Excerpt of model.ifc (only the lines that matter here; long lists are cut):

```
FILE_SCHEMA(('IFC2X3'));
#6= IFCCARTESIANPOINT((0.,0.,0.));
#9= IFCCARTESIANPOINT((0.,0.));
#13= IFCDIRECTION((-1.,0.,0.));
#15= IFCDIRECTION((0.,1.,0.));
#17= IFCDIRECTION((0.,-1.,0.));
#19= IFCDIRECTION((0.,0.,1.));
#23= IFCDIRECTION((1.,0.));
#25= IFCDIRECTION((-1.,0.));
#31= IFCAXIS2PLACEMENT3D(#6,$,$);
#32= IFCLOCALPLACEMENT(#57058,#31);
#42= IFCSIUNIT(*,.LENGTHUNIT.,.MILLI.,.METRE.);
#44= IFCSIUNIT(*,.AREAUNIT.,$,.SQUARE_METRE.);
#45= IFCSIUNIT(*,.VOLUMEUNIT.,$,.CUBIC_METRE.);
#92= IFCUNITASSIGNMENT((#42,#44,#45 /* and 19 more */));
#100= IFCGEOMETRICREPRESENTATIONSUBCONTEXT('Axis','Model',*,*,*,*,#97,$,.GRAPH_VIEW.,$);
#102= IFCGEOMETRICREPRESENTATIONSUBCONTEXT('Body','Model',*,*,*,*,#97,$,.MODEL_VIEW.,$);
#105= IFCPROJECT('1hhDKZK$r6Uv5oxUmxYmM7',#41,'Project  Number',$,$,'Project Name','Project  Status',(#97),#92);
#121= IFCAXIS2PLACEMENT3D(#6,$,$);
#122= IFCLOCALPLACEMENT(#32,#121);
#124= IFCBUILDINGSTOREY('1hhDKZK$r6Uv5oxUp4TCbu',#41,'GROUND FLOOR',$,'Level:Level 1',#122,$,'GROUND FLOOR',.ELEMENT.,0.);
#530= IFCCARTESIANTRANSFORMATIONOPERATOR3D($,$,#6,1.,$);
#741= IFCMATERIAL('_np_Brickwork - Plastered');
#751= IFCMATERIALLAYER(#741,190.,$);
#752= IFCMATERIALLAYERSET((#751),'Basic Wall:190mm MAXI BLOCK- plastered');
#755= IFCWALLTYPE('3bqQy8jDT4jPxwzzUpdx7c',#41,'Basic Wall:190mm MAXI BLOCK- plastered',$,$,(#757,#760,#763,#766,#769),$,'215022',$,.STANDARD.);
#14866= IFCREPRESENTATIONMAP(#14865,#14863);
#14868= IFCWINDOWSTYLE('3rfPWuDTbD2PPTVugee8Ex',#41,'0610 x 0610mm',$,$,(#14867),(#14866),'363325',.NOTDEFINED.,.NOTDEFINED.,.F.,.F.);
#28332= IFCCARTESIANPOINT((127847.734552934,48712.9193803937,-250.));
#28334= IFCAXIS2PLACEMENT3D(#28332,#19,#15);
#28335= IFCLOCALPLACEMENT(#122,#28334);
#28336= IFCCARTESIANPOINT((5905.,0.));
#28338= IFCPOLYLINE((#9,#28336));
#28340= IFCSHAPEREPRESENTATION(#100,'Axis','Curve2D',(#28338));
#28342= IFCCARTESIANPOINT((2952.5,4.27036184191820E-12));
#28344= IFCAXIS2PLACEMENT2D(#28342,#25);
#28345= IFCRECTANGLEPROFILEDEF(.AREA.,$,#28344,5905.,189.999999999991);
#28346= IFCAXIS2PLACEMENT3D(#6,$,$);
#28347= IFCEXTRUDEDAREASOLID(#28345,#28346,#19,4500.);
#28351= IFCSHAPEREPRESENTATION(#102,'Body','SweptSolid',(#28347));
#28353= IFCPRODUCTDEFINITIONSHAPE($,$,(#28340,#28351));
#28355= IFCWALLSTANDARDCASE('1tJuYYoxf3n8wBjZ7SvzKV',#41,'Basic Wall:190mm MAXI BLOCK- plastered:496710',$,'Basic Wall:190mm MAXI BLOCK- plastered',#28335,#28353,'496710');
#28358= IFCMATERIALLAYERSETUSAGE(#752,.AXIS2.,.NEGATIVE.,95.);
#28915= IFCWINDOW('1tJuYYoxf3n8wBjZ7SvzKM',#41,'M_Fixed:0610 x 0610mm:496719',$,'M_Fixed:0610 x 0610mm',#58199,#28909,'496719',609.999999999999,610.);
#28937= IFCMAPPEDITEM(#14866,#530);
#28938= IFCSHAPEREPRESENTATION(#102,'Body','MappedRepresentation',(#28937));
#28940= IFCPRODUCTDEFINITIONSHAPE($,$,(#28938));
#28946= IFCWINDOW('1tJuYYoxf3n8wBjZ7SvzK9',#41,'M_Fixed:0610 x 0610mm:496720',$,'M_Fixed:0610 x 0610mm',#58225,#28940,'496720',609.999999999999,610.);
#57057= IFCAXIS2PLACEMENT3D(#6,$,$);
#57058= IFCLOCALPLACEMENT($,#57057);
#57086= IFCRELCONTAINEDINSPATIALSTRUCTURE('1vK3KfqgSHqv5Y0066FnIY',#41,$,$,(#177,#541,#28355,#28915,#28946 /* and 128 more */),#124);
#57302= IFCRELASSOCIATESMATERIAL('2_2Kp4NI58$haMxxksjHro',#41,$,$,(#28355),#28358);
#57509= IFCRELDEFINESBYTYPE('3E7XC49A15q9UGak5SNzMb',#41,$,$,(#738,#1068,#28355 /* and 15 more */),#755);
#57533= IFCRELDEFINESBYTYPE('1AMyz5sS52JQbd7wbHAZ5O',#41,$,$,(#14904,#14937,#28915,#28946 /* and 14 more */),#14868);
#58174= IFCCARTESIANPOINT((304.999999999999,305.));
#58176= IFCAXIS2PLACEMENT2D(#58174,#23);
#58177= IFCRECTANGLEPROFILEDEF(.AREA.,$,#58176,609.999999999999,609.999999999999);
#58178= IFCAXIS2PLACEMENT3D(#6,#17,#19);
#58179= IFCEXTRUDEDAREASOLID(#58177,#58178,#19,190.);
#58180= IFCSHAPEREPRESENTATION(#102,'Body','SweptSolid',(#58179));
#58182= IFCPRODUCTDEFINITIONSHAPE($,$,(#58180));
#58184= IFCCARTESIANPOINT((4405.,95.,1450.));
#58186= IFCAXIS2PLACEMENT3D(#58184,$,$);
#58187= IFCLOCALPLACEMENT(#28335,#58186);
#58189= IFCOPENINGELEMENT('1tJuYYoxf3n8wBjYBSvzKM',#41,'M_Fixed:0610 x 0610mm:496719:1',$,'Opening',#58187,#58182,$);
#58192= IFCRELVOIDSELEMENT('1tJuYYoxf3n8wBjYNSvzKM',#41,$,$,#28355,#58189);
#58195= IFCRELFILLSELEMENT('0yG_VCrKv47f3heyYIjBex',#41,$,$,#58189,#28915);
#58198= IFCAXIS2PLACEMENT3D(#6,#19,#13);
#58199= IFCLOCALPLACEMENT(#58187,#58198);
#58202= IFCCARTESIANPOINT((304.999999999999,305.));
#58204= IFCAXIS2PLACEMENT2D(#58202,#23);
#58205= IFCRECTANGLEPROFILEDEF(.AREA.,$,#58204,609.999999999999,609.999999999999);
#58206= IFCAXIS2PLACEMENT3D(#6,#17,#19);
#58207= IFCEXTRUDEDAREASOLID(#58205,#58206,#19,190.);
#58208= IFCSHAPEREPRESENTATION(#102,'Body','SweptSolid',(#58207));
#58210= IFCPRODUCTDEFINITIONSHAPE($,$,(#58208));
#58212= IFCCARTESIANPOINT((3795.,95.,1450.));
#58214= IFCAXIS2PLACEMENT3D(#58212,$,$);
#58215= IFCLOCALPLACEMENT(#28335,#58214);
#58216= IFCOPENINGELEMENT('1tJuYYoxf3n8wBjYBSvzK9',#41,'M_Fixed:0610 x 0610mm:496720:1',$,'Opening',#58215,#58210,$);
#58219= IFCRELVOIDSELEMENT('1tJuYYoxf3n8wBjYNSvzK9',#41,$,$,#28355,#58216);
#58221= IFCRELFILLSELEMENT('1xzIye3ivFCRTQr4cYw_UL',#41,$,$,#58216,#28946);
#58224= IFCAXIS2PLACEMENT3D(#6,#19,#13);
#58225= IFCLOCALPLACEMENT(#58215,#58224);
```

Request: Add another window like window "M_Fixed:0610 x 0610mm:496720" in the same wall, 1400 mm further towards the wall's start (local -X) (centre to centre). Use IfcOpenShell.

```python
import ifcopenshell
import ifcopenshell.api.feature
import ifcopenshell.api.geometry
import ifcopenshell.api.root
import ifcopenshell.geom
import ifcopenshell.util.element
import ifcopenshell.util.placement
import ifcopenshell.util.shape

model = ifcopenshell.open("model.ifc")
settings = ifcopenshell.geom.settings()


def volume(element):
    """Net volume in cubic metres, openings subtracted."""
    shape = ifcopenshell.geom.create_shape(settings, element)
    return ifcopenshell.util.shape.get_volume(shape.geometry)


def reuse_history(source, copy):
    """copy_class also copies each property set's owner history, people and application; keep the originals."""
    for rel in copy.IsDefinedBy:
        if rel.is_a("IfcRelDefinesByProperties") and (history := rel.RelatingPropertyDefinition.OwnerHistory):
            rel.RelatingPropertyDefinition.OwnerHistory = source.OwnerHistory
            ifcopenshell.util.element.remove_deep2(model, history)


window = model.by_guid("1tJuYYoxf3n8wBjZ7SvzK9")
opening = window.FillsVoids[0].RelatingOpeningElement
wall = opening.VoidsElements[0].RelatingBuildingElement
before = volume(wall)
shift = ifcopenshell.util.placement.get_local_placement(wall.ObjectPlacement)[:3, 0] * -1400.0

# copy_class copies the void relationship, type, container and properties, but no geometry.
new_opening = ifcopenshell.api.root.copy_class(model, product=opening)
new_opening.Representation = ifcopenshell.util.element.copy_deep(
    model, opening.Representation, exclude=["IfcGeometricRepresentationContext", "IfcRepresentationMap"]
)
new_opening.Name = "M_Fixed:0610 x 0610mm"
new_window = ifcopenshell.api.root.copy_class(model, product=window)
new_window.Representation = ifcopenshell.util.element.copy_deep(
    model, window.Representation, exclude=["IfcGeometricRepresentationContext", "IfcRepresentationMap"]
)
new_window.Name = "M_Fixed:0610 x 0610mm"
new_window.Tag = None
reuse_history(window, new_window)
fills = ifcopenshell.api.feature.add_filling(model, opening=new_opening, element=new_window)
fills.OwnerHistory = new_window.OwnerHistory  # required in IFC2X3

for old, new in ((opening, new_opening), (window, new_window)):
    matrix = ifcopenshell.util.placement.get_local_placement(old.ObjectPlacement)
    matrix[:3, 3] += shift
    ifcopenshell.api.geometry.edit_object_placement(model, product=new, matrix=matrix, is_si=False)

after = volume(wall)

print(f"wall volume {before:.3f} -> {after:.3f} m3")

model.write("model-out.ifc")
```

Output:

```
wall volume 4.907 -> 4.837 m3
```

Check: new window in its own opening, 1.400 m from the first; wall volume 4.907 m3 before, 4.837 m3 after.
